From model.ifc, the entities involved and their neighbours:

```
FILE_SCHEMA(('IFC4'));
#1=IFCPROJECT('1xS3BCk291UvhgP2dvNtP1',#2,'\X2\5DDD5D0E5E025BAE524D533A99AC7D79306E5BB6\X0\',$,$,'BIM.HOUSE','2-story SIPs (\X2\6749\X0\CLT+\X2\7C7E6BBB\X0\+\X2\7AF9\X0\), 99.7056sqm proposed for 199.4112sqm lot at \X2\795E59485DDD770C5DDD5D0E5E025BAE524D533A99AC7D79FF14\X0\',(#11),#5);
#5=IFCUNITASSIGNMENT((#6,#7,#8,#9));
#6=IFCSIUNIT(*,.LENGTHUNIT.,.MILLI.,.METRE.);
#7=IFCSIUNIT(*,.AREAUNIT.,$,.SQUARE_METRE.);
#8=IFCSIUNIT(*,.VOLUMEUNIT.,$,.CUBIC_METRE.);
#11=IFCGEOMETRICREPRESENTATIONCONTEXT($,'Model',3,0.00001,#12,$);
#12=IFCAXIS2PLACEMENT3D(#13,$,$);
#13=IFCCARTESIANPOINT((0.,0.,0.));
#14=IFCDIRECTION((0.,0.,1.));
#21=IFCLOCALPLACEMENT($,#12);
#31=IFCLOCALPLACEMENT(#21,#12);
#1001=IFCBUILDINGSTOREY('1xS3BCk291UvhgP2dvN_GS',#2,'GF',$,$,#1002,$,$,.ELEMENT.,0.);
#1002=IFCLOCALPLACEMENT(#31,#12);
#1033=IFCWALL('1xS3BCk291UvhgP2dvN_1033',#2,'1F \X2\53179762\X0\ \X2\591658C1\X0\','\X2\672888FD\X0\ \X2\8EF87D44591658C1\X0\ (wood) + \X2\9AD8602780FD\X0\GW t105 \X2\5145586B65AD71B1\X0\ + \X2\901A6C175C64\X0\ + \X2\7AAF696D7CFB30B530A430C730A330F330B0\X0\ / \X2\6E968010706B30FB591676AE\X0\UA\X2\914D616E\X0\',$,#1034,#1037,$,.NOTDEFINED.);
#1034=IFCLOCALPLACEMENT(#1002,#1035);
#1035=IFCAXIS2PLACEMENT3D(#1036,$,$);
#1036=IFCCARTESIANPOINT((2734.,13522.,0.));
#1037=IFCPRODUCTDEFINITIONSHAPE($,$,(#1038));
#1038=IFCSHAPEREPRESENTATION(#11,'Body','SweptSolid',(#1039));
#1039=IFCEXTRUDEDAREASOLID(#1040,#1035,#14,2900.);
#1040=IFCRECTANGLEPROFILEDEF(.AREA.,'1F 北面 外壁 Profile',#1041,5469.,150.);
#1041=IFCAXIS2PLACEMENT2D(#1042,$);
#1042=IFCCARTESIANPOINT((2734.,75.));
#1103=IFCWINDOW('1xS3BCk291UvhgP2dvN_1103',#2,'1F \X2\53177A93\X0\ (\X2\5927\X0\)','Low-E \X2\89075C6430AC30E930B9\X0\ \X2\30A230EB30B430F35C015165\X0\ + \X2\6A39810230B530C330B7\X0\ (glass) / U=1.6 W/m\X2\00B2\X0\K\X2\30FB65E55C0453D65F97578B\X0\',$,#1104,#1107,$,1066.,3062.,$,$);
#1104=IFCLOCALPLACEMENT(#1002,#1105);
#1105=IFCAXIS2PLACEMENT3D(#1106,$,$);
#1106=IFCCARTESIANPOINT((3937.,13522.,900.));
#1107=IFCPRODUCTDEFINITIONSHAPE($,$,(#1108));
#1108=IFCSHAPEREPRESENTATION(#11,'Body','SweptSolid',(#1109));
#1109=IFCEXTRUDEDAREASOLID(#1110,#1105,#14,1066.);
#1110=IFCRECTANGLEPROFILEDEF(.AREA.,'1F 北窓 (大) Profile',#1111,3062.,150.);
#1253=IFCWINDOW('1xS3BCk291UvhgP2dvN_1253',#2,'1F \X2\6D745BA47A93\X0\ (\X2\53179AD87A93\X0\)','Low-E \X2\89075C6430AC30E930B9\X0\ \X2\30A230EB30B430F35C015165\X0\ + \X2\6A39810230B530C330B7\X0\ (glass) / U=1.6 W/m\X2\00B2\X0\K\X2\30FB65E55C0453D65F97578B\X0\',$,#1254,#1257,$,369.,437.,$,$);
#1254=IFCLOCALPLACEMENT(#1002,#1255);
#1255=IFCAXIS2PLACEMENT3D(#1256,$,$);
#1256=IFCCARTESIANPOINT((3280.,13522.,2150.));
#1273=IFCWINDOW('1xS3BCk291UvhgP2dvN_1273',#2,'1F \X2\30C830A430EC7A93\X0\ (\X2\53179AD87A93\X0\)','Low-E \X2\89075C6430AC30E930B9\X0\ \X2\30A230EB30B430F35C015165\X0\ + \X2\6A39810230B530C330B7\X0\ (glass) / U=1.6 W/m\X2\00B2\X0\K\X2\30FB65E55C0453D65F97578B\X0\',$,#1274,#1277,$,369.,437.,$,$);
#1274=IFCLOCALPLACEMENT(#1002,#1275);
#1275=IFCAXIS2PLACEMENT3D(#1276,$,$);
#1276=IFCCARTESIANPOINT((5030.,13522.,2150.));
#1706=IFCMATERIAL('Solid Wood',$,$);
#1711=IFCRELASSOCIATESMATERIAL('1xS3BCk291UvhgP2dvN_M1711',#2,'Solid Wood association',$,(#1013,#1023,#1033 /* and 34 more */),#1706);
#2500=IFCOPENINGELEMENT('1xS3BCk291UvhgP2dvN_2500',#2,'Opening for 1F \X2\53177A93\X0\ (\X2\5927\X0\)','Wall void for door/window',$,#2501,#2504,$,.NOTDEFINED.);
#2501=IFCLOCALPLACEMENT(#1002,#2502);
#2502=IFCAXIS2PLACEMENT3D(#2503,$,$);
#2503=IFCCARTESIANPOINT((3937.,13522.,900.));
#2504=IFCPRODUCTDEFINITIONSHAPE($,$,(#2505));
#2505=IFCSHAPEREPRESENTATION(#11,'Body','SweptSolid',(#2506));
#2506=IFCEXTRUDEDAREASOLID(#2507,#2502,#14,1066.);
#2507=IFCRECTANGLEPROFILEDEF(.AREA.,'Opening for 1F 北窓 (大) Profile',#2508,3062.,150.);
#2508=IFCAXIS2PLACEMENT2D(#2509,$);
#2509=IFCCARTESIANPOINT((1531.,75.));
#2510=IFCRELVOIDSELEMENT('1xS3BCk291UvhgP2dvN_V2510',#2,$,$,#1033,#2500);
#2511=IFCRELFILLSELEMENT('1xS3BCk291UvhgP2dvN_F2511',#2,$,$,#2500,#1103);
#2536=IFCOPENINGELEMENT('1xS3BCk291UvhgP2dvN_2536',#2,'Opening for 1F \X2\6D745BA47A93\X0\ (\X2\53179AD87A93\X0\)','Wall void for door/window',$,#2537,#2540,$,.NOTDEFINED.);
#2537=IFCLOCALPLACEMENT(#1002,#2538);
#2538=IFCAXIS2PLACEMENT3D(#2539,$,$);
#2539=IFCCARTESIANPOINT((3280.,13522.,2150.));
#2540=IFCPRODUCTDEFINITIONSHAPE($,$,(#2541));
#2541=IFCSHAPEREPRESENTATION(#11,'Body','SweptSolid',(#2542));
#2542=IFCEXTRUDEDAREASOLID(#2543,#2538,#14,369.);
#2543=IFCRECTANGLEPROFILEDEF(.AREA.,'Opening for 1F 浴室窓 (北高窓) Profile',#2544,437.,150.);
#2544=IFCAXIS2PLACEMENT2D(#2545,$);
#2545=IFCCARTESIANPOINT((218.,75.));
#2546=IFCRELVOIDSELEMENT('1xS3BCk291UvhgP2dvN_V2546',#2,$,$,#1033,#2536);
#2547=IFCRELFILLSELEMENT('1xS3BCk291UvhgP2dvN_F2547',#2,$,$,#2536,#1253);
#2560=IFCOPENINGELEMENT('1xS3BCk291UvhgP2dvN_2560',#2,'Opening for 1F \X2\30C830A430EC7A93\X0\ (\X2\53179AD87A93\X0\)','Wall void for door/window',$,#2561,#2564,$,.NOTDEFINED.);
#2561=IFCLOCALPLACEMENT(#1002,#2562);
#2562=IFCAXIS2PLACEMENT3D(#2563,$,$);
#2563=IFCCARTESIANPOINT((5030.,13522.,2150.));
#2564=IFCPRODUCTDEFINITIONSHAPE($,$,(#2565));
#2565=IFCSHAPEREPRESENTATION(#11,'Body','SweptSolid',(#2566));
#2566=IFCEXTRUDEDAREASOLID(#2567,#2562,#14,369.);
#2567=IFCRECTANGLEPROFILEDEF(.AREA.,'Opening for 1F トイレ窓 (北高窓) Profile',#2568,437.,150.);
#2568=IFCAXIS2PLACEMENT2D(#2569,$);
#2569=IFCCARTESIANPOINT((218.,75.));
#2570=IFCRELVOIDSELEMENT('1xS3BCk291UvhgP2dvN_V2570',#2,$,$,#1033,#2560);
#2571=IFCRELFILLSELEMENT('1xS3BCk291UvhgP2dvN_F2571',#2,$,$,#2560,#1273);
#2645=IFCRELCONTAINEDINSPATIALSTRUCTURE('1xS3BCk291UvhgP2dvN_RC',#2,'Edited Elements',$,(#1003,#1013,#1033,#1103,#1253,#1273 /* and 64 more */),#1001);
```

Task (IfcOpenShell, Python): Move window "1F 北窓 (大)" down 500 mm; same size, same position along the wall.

```python
import numpy as np
import ifcopenshell
import ifcopenshell.api.geometry
import ifcopenshell.util.placement
import ifcopenshell.util.unit

model = ifcopenshell.open("model.ifc")
unit_scale = ifcopenshell.util.unit.calculate_unit_scale(model)

window = model.by_id(1103)
opening = window.FillsVoids[0].RelatingOpeningElement
dz = -0.5 / unit_scale

shift = np.array([0.0, 0.0, dz])
# The window is not placed relative to its opening, so move both.
for product in (opening, window):
    matrix = ifcopenshell.util.placement.get_local_placement(product.ObjectPlacement)
    matrix[:3, 3] += shift
    ifcopenshell.api.geometry.edit_object_placement(model, product=product, matrix=matrix, is_si=False)

print(f"moved by {dz * unit_scale:+.3f} m")

model.write("model-out.ifc")
```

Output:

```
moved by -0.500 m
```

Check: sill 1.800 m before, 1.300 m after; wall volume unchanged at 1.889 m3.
